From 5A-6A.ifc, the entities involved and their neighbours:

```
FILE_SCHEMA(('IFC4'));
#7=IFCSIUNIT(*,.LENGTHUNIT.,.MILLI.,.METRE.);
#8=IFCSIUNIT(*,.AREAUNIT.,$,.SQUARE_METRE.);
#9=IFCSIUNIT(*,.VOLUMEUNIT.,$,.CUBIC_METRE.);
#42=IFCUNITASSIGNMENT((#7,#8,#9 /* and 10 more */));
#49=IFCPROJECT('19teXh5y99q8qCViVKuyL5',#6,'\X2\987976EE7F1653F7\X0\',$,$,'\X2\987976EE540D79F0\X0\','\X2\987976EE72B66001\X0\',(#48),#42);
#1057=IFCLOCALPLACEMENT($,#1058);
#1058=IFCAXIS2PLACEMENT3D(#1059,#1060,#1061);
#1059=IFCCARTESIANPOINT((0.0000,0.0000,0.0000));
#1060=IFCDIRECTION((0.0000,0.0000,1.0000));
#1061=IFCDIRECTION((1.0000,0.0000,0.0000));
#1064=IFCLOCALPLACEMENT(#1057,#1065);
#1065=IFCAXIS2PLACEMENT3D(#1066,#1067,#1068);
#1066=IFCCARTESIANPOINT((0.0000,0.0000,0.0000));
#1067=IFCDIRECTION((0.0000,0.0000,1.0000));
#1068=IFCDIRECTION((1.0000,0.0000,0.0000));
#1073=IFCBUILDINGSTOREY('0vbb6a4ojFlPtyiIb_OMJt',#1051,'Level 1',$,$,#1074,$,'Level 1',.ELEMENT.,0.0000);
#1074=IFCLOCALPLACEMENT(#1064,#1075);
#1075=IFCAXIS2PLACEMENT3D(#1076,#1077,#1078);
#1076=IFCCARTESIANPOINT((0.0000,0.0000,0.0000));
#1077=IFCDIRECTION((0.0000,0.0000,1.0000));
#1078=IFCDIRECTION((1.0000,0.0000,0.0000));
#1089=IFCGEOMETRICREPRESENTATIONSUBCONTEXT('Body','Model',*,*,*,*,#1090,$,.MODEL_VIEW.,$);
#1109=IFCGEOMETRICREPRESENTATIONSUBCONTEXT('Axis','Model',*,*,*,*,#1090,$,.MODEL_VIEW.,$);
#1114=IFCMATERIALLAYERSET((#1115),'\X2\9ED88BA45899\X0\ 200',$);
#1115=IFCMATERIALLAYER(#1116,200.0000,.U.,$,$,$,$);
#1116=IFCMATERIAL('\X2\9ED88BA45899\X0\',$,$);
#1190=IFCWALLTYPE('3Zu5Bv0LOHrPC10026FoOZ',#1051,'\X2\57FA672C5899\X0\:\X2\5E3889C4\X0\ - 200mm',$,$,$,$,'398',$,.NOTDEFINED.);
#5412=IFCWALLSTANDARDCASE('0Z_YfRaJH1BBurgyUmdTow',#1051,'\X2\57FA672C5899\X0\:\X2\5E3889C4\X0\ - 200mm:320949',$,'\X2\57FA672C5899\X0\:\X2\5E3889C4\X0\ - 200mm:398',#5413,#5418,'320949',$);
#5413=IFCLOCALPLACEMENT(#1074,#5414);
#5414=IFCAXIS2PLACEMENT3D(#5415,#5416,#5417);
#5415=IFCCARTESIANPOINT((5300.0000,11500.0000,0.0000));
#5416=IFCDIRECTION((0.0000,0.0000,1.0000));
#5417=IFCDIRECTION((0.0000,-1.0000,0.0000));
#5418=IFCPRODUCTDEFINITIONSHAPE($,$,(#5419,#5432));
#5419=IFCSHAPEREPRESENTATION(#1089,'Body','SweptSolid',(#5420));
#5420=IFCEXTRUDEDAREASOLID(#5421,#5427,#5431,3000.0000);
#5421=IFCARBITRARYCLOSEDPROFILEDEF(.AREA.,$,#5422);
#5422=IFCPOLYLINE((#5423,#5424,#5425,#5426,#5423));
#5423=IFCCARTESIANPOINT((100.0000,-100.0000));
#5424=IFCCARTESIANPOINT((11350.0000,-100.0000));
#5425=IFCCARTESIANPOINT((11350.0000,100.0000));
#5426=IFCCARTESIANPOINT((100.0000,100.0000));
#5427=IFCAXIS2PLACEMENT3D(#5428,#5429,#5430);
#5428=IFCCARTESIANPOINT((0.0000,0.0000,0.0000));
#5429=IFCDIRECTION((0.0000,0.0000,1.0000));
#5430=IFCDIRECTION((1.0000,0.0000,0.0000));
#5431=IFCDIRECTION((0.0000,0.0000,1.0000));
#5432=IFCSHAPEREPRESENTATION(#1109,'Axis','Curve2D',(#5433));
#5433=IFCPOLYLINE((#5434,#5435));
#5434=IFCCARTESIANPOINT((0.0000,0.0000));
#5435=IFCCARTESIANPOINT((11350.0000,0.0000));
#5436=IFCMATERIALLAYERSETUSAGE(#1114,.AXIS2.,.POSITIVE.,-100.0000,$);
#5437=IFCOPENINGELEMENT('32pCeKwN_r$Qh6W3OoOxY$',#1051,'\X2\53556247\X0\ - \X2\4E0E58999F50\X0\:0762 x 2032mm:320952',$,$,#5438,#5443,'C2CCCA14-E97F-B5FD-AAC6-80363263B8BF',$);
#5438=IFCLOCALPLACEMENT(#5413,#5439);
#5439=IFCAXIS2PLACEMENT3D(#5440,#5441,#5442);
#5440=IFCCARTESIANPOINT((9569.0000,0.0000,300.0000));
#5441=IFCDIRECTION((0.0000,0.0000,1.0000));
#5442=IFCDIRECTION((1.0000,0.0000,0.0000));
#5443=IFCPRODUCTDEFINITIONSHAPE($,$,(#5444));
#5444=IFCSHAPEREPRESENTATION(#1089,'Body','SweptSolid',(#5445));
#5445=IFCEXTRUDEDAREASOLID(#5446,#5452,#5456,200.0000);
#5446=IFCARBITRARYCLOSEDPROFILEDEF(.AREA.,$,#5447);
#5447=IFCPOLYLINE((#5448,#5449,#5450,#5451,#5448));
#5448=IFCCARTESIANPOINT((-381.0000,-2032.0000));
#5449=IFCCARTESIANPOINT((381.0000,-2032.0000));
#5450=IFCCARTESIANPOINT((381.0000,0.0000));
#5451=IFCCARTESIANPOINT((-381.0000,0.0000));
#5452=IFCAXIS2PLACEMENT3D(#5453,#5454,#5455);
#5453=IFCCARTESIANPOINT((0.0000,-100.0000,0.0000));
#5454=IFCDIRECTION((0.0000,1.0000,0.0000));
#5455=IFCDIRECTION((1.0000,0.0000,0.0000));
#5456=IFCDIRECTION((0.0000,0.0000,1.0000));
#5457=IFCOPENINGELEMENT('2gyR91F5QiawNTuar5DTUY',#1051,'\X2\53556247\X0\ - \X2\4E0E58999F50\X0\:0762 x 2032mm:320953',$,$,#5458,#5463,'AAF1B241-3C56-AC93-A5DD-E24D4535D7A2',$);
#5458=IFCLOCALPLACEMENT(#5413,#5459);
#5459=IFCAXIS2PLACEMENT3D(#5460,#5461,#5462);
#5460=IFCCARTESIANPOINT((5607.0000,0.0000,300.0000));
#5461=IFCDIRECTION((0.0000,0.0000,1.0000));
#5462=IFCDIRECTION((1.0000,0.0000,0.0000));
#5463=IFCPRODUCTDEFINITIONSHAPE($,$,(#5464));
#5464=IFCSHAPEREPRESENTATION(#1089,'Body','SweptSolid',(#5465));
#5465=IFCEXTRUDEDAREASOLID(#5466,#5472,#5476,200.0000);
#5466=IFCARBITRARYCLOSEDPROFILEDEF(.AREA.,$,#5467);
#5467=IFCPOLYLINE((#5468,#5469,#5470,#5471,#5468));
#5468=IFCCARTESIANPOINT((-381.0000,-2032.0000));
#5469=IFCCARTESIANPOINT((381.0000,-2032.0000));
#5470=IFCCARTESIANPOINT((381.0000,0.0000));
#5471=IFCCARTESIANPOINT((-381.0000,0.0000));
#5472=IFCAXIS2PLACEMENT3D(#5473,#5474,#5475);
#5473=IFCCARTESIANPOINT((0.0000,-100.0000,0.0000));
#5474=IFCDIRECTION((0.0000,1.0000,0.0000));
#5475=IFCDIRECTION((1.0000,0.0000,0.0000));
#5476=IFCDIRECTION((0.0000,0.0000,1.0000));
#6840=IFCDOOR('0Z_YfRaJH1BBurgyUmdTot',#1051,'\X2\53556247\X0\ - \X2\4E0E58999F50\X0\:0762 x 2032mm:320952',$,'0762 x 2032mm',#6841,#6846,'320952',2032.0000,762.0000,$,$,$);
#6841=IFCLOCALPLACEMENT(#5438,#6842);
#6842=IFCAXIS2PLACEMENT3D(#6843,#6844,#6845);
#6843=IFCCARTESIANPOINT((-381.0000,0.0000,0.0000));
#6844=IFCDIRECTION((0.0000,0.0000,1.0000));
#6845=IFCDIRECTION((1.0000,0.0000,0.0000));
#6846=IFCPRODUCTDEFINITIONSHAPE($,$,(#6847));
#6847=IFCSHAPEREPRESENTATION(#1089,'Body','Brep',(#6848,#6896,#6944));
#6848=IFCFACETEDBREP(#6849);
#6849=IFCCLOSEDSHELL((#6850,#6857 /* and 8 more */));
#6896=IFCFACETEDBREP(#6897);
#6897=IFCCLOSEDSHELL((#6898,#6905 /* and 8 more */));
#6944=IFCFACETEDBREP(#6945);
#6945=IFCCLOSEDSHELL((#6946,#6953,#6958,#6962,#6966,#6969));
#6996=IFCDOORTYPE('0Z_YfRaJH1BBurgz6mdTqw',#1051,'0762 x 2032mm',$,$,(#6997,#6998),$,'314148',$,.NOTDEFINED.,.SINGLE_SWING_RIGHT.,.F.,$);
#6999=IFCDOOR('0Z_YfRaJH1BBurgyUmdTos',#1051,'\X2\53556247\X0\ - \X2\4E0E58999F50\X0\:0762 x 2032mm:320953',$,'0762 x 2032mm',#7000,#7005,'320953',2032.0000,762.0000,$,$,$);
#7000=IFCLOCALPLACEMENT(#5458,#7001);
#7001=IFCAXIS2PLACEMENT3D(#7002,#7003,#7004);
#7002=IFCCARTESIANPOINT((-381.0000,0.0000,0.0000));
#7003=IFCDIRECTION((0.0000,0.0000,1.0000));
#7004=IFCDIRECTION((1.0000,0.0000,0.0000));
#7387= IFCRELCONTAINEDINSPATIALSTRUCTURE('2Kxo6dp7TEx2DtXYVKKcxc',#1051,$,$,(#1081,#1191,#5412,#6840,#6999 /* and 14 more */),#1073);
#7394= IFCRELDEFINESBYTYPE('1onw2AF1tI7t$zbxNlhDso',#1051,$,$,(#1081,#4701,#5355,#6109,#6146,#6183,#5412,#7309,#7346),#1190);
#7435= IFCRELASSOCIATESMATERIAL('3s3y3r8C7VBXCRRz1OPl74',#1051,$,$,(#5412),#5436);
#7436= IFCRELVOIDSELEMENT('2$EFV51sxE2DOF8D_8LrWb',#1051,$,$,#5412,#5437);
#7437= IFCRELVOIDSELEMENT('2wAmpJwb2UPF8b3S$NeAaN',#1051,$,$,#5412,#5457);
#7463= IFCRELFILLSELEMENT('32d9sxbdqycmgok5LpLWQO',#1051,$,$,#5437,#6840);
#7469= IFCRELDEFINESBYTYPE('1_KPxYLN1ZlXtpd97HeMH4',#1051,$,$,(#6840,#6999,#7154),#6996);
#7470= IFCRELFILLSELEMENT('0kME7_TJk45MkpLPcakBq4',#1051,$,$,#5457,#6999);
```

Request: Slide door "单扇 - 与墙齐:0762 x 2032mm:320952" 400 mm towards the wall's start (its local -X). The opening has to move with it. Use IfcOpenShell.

```python
import ifcopenshell
import ifcopenshell.api.geometry
import ifcopenshell.util.placement

model = ifcopenshell.open("5A-6A.ifc")

door = model.by_guid("0Z_YfRaJH1BBurgyUmdTot")
opening = door.FillsVoids[0].RelatingOpeningElement
wall = opening.VoidsElements[0].RelatingBuildingElement

wall_matrix = ifcopenshell.util.placement.get_local_placement(wall.ObjectPlacement)
shift = wall_matrix[:3, 0] * -400.0
before = ifcopenshell.util.placement.get_local_placement(door.ObjectPlacement)[:3, 3].copy()

# The door is placed relative to its opening, so it follows when the opening moves.
matrix = ifcopenshell.util.placement.get_local_placement(opening.ObjectPlacement)
matrix[:3, 3] += shift
ifcopenshell.api.geometry.edit_object_placement(
    model, product=opening, matrix=matrix, is_si=False, should_transform_children=True
)

after = ifcopenshell.util.placement.get_local_placement(door.ObjectPlacement)[:3, 3]
print("door moved by", (after - before).round(3) + 0.0)

model.write("5A-6A_edited.ifc")
```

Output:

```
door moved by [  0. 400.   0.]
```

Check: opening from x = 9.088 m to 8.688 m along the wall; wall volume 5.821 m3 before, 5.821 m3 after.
